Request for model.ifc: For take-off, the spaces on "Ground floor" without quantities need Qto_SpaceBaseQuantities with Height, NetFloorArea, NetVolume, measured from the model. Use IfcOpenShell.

First a look at what the model holds.

```python
import ifcopenshell
import ifcopenshell.util.element
import ifcopenshell.util.unit

model = ifcopenshell.open("model.ifc")
print(model.schema)
for unit_type in ("LENGTHUNIT", "AREAUNIT", "VOLUMEUNIT"):
    print(unit_type, ifcopenshell.util.unit.calculate_unit_scale(model, unit_type))
storey = next(s for s in model.by_type("IfcBuildingStorey") if s.Name == "Ground floor")
spaces = [e for e in ifcopenshell.util.element.get_decomposition(storey) if e.is_a("IfcSpace")]
for e in sorted(spaces, key=lambda e: e.id()):
    print(e.id(), e.is_a(), e.Name, list(ifcopenshell.util.element.get_psets(e, qtos_only=True)), sep=" | ")
```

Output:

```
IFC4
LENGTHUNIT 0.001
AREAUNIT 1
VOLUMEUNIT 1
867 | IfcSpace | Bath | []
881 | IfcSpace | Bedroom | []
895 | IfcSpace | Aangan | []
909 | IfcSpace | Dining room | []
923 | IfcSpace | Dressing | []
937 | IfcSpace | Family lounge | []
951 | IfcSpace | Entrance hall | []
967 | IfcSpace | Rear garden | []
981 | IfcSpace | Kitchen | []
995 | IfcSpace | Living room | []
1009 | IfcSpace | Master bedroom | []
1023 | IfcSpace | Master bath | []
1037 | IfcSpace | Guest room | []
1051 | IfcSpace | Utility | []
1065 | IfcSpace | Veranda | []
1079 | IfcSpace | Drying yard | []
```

```python
import ifcopenshell
import ifcopenshell.api.pset
import ifcopenshell.geom
import ifcopenshell.util.element
import ifcopenshell.util.shape
import ifcopenshell.util.unit

model = ifcopenshell.open("model.ifc")
unit_scale = ifcopenshell.util.unit.calculate_unit_scale(model)
area_scale = ifcopenshell.util.unit.calculate_unit_scale(model, "AREAUNIT")
volume_scale = ifcopenshell.util.unit.calculate_unit_scale(model, "VOLUMEUNIT")
settings = ifcopenshell.geom.settings()

storey = next(s for s in model.by_type("IfcBuildingStorey") if s.Name == "Ground floor")
spaces = [e for e in ifcopenshell.util.element.get_decomposition(storey) if e.is_a("IfcSpace")]

for e in sorted(spaces, key=lambda e: e.id()):
    if ifcopenshell.util.element.get_psets(e, qtos_only=True, should_inherit=False):
        continue
    # Geometry comes back in metres, in the element's own axes.
    shape = ifcopenshell.geom.create_shape(settings, e)
    values = {
        "Height": ifcopenshell.util.shape.get_z(shape.geometry) / unit_scale,
        "NetFloorArea": ifcopenshell.util.shape.get_footprint_area(shape.geometry) / area_scale,
        "NetVolume": ifcopenshell.util.shape.get_volume(shape.geometry) / volume_scale,
    }
    qto = ifcopenshell.api.pset.add_qto(model, product=e, name="Qto_SpaceBaseQuantities")
    ifcopenshell.api.pset.edit_qto(model, qto=qto, properties=values)
    print(e.id(), {k: round(v, 3) for k, v in values.items()})

model.write("model_rev.ifc")
```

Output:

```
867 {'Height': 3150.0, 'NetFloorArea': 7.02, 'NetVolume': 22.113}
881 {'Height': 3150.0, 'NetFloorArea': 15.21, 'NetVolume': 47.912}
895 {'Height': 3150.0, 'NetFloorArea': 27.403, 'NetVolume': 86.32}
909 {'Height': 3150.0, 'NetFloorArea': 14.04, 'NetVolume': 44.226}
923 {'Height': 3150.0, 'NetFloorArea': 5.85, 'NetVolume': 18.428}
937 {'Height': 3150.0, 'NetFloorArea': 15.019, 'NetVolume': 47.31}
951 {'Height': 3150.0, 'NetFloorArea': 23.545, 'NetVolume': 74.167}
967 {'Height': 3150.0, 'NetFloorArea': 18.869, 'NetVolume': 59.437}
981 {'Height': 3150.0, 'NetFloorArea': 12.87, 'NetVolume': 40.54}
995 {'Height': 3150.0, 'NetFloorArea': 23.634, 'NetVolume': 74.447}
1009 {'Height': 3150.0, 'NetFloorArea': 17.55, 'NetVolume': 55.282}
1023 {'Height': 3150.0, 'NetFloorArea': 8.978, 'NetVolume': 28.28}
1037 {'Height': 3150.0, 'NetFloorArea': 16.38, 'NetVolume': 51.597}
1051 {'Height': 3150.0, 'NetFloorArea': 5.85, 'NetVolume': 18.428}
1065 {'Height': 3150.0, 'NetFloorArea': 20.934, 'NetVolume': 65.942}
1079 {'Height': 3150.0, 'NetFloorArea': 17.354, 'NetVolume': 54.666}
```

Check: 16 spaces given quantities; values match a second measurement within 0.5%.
